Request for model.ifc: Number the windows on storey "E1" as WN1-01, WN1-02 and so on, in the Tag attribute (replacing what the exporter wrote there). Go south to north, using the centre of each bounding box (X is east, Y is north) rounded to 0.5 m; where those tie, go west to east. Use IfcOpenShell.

First a look at what the model holds.

```python
import ifcopenshell
import ifcopenshell.util.element
import ifcopenshell.util.placement

model = ifcopenshell.open("model.ifc")
print(model.schema)
storey = next(s for s in model.by_type("IfcBuildingStorey") if s.Name == "E1")
windows = [e for e in ifcopenshell.util.element.get_decomposition(storey) if e.is_a("IfcWindow")]
for e in sorted(windows, key=lambda e: e.id()):
    origin = ifcopenshell.util.placement.get_local_placement(e.ObjectPlacement)[:3, 3]
    print(e.id(), e.Tag, e.Name, origin.round(2) + 0.0, sep=" | ")
```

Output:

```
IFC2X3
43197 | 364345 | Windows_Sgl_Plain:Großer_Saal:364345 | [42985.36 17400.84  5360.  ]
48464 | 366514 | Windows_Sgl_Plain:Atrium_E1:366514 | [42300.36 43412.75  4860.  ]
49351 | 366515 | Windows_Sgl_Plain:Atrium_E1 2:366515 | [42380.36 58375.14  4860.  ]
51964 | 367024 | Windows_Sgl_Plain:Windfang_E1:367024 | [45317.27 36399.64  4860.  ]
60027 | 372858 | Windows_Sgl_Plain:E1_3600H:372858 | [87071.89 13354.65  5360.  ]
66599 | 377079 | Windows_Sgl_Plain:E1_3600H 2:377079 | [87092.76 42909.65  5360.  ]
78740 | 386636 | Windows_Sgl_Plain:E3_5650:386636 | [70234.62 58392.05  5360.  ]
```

```python
import ifcopenshell
import ifcopenshell.geom
import ifcopenshell.util.element
import ifcopenshell.util.shape

model = ifcopenshell.open("model.ifc")
settings = ifcopenshell.geom.settings()
settings.set("use-world-coords", True)


def centre(element):
    shape = ifcopenshell.geom.create_shape(settings, element)
    return ifcopenshell.util.shape.get_bbox_centroid(shape.geometry)


storey = next(s for s in model.by_type("IfcBuildingStorey") if s.Name == "E1")
windows = [e for e in ifcopenshell.util.element.get_decomposition(storey) if e.is_a("IfcWindow")]

# Insertion points can sit at a corner or the storey origin, so sort by the geometry (in metres).
centres = {e: centre(e) for e in windows}
windows.sort(key=lambda e: (round(centres[e][1] / 0.5), centres[e][0]))

for i, e in enumerate(windows, start=1):
    number = f"WN1-{i:02d}"
    e.Tag = number
    print(e.id(), number)

model.write("model_updated.ifc")
```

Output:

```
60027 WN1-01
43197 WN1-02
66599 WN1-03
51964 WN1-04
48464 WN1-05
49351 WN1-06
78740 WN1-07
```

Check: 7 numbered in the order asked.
